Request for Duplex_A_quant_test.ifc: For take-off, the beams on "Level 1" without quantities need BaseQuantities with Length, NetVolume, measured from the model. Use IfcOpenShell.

First a look at what the model holds.

```python
import ifcopenshell
import ifcopenshell.util.element
import ifcopenshell.util.unit

model = ifcopenshell.open("Duplex_A_quant_test.ifc")
print(model.schema)
for unit_type in ("LENGTHUNIT", "AREAUNIT", "VOLUMEUNIT"):
    print(unit_type, ifcopenshell.util.unit.calculate_unit_scale(model, unit_type))
storey = next(s for s in model.by_type("IfcBuildingStorey") if s.Name == "Level 1")
beams = [e for e in ifcopenshell.util.element.get_decomposition(storey) if e.is_a("IfcBeam")]
for e in sorted(beams, key=lambda e: e.id()):
    print(e.id(), e.is_a(), e.Name, list(ifcopenshell.util.element.get_psets(e, qtos_only=True)), sep=" | ")
```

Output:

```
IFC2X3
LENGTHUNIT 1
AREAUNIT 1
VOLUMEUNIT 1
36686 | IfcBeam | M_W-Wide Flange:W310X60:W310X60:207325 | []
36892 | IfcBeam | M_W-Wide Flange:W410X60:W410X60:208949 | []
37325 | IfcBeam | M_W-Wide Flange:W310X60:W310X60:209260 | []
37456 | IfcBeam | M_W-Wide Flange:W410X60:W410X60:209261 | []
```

```python
import ifcopenshell
import ifcopenshell.api.pset
import ifcopenshell.geom
import ifcopenshell.util.element
import ifcopenshell.util.shape
import ifcopenshell.util.unit

model = ifcopenshell.open("Duplex_A_quant_test.ifc")
unit_scale = ifcopenshell.util.unit.calculate_unit_scale(model)
volume_scale = ifcopenshell.util.unit.calculate_unit_scale(model, "VOLUMEUNIT")
settings = ifcopenshell.geom.settings()

storey = next(s for s in model.by_type("IfcBuildingStorey") if s.Name == "Level 1")
beams = [e for e in ifcopenshell.util.element.get_decomposition(storey) if e.is_a("IfcBeam")]

for e in sorted(beams, key=lambda e: e.id()):
    if ifcopenshell.util.element.get_psets(e, qtos_only=True, should_inherit=False):
        continue
    # Geometry comes back in metres, in the element's own axes.
    shape = ifcopenshell.geom.create_shape(settings, e)
    values = {
        "Length": ifcopenshell.util.shape.get_max_xyz(shape.geometry) / unit_scale,
        "NetVolume": ifcopenshell.util.shape.get_volume(shape.geometry) / volume_scale,
    }
    qto = ifcopenshell.api.pset.add_qto(model, product=e, name="BaseQuantities")
    ifcopenshell.api.pset.edit_qto(model, qto=qto, properties=values)
    print(e.id(), {k: round(v, 3) for k, v in values.items()})

model.write("Duplex_A_quant_test_v2.ifc")
```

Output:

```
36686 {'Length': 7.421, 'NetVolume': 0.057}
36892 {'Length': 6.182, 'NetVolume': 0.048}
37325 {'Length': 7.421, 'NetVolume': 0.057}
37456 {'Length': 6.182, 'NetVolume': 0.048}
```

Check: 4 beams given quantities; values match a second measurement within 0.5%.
